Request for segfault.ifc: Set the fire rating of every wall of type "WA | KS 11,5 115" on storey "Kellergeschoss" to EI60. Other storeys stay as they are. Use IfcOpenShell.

First a look at what the model holds.

```python
import ifcopenshell
import ifcopenshell.util.element

model = ifcopenshell.open("segfault.ifc")
print(model.schema)
storey = next(s for s in model.by_type("IfcBuildingStorey") if s.Name == "Kellergeschoss")
walls = [e for e in ifcopenshell.util.element.get_decomposition(storey) if e.is_a("IfcWall")]
seen = {}
for e in walls:
    element_type = ifcopenshell.util.element.get_type(e)
    key = (element_type.Name if element_type != e and element_type else None, ifcopenshell.util.element.get_pset(e, "Pset_WallCommon", "FireRating"))
    seen[key] = seen.get(key, 0) + 1
for (name, value), count in sorted(seen.items(), key=str):
    print(count, "x", name, "|", value)
```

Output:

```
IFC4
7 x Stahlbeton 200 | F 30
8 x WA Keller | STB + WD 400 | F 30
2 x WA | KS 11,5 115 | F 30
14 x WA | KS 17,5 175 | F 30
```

```python
import ifcopenshell
import ifcopenshell.api.pset
import ifcopenshell.util.element

model = ifcopenshell.open("segfault.ifc")

storey = next(s for s in model.by_type("IfcBuildingStorey") if s.Name == "Kellergeschoss")
walls = [e for e in ifcopenshell.util.element.get_decomposition(storey) if e.is_a("IfcWall")]

count = 0
for e in walls:
    element_type = ifcopenshell.util.element.get_type(e)
    if element_type in (None, e) or element_type.Name != 'WA\xa0|\xa0KS 11,5 115':
        continue
    # add_pset returns the element's existing set when there is one.
    pset = ifcopenshell.api.pset.add_pset(model, product=e, name="Pset_WallCommon")
    ifcopenshell.api.pset.edit_pset(model, pset=pset, properties={"FireRating": "EI60"})
    count += 1

print(count, "walls updated")

model.write("segfault_updated.ifc")
```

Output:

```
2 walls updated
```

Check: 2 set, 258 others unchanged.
